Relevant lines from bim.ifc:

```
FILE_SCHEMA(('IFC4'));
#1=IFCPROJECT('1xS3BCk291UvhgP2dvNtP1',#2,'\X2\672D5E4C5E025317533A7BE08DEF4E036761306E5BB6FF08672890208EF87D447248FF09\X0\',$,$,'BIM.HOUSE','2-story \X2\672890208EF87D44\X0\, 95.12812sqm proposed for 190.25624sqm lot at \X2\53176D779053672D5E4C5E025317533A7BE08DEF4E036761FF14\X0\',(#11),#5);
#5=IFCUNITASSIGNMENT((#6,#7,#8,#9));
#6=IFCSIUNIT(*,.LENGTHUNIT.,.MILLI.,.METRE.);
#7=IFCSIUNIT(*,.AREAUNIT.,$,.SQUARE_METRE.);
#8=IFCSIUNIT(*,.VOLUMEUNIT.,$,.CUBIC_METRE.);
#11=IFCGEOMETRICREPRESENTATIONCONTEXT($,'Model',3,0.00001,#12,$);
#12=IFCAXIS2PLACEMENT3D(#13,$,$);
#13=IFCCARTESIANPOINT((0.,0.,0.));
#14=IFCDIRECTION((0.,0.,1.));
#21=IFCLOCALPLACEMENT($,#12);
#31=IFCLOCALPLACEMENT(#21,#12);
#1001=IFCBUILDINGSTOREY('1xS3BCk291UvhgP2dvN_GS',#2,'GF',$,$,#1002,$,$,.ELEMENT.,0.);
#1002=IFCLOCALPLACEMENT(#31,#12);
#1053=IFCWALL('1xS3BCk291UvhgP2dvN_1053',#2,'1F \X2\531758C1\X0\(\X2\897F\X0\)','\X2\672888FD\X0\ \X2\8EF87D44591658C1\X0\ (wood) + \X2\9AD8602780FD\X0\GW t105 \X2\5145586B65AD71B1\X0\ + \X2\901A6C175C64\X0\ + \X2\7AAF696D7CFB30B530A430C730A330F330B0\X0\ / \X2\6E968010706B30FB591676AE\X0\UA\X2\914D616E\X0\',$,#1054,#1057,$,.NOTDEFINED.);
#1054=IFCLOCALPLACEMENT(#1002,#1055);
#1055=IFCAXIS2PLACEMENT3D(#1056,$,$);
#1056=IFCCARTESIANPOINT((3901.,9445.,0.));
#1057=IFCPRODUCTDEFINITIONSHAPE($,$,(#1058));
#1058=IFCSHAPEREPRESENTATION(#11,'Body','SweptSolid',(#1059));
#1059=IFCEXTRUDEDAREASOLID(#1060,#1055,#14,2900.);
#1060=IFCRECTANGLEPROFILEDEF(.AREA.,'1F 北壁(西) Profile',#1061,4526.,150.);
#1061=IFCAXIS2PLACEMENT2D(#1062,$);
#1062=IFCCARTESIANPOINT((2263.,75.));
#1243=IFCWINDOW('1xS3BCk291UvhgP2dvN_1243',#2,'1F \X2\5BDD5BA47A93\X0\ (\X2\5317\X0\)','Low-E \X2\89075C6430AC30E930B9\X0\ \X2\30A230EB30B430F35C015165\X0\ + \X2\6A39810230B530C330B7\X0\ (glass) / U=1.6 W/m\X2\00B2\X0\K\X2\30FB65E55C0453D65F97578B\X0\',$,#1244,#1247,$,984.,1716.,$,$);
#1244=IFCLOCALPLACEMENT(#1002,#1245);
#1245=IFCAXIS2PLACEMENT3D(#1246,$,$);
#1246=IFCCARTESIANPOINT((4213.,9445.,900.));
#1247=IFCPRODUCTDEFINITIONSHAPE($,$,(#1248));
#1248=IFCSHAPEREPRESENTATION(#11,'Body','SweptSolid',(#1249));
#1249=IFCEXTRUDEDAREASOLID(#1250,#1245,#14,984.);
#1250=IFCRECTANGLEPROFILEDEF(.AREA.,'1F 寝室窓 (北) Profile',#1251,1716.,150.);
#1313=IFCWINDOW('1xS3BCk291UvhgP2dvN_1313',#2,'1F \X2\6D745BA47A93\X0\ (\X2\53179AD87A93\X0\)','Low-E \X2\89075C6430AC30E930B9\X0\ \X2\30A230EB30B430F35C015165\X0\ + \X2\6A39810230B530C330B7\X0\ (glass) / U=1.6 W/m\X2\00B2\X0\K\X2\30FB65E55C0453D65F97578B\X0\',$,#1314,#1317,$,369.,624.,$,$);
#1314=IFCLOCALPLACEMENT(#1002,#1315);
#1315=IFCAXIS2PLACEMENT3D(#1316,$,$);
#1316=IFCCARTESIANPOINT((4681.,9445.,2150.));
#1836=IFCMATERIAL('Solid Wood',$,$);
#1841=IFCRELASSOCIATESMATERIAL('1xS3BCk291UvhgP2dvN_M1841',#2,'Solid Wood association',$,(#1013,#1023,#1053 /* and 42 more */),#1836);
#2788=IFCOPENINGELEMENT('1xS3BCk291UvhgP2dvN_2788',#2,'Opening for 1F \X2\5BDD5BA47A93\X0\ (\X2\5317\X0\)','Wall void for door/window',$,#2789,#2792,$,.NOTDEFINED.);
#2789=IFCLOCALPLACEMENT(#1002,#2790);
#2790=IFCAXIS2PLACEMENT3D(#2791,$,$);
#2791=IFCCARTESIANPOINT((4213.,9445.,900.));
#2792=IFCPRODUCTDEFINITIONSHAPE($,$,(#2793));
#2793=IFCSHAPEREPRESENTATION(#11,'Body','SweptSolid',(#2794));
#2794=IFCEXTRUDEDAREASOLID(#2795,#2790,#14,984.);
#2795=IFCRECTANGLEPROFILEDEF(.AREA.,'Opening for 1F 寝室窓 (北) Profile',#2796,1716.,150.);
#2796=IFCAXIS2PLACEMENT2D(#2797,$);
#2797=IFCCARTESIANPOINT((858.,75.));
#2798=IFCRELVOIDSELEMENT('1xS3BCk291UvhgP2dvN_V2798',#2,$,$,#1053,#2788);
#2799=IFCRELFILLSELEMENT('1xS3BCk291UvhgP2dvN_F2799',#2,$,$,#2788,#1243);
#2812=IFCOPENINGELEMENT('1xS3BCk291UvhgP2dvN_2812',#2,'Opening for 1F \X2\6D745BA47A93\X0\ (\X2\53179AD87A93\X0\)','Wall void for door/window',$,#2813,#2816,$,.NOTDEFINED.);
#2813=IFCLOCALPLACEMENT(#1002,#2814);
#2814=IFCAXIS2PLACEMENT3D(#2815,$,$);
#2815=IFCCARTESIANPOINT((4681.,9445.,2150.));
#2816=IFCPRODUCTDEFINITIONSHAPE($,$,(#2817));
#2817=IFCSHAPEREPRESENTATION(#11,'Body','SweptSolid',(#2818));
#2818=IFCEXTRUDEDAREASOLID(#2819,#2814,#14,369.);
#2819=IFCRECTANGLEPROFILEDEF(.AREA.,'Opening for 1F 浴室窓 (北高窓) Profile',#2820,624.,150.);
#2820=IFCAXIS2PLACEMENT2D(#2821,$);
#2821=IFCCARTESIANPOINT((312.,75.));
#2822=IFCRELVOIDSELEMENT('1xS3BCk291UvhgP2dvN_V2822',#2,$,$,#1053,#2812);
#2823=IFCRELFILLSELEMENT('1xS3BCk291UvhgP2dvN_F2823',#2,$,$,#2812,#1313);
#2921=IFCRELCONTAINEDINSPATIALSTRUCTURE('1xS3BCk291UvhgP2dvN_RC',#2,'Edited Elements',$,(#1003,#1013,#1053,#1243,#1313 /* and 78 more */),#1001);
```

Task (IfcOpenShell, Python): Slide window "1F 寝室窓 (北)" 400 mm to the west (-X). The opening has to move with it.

```python
import ifcopenshell
import ifcopenshell.api.geometry
import ifcopenshell.util.placement
import ifcopenshell.util.unit

model = ifcopenshell.open("bim.ifc")
unit_scale = ifcopenshell.util.unit.calculate_unit_scale(model)

window = model.by_id(1243)
opening = window.FillsVoids[0].RelatingOpeningElement
wall = opening.VoidsElements[0].RelatingBuildingElement

wall_matrix = ifcopenshell.util.placement.get_local_placement(wall.ObjectPlacement)
shift = wall_matrix[:3, 0] * -0.4 / unit_scale
before = ifcopenshell.util.placement.get_local_placement(window.ObjectPlacement)[:3, 3].copy()

# The window is not placed relative to its opening, so move both.
for product in (opening, window):
    matrix = ifcopenshell.util.placement.get_local_placement(product.ObjectPlacement)
    matrix[:3, 3] += shift
    ifcopenshell.api.geometry.edit_object_placement(model, product=product, matrix=matrix, is_si=False)

after = ifcopenshell.util.placement.get_local_placement(window.ObjectPlacement)[:3, 3]
print("window moved by", (after - before).round(3) + 0.0)

model.write("bim-out.ifc")
```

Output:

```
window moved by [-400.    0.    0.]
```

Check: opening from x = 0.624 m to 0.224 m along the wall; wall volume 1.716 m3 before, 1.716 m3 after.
